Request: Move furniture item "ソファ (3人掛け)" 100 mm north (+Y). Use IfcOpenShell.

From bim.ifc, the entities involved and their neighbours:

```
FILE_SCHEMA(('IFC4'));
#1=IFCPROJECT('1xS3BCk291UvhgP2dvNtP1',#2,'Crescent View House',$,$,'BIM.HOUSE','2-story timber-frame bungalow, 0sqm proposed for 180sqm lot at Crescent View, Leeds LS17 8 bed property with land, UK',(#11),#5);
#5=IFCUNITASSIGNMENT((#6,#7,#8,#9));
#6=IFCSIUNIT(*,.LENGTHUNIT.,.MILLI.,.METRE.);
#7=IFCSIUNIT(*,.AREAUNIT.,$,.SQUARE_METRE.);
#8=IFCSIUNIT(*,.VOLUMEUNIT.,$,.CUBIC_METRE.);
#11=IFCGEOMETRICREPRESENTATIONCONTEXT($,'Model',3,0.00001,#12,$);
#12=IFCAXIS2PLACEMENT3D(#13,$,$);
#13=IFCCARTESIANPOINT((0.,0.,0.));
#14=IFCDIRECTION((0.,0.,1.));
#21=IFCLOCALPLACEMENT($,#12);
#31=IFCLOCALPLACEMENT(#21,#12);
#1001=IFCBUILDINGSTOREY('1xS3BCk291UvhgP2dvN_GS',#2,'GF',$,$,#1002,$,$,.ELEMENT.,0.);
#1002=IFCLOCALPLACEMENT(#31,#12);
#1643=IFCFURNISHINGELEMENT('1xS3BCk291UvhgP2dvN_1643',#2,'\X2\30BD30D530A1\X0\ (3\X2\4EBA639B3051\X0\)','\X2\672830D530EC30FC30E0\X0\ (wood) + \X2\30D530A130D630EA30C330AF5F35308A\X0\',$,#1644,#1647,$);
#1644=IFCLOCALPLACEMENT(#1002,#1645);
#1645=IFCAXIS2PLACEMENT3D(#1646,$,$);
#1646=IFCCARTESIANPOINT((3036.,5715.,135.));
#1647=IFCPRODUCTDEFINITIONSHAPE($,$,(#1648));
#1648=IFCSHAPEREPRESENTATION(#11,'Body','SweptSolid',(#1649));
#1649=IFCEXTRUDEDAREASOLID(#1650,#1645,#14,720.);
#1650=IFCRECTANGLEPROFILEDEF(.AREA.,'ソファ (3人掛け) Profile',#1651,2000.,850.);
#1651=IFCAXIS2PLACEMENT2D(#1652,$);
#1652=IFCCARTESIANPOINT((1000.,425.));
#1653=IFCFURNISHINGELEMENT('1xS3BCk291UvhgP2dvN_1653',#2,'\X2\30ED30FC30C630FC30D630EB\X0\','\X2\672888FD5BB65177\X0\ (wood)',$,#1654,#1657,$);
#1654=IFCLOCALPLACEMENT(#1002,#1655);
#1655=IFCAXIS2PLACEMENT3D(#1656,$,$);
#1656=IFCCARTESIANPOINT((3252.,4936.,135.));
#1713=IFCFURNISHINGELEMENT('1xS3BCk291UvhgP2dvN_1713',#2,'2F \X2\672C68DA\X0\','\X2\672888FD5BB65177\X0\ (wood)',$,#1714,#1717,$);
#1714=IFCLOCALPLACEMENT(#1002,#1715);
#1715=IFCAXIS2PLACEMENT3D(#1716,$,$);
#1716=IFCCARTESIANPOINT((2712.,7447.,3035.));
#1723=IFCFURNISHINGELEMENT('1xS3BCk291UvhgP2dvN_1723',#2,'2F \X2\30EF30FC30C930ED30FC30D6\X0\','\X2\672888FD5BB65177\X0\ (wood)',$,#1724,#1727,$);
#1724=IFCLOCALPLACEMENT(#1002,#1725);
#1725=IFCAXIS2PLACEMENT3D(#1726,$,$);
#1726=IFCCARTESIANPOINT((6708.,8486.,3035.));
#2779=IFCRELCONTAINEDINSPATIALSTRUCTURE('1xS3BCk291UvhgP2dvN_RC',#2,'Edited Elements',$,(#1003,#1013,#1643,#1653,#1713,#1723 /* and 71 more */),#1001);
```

```python
import ifcopenshell
import ifcopenshell.api.geometry
import ifcopenshell.util.placement
import ifcopenshell.util.unit

model = ifcopenshell.open("bim.ifc")
unit_scale = ifcopenshell.util.unit.calculate_unit_scale(model)

item = model.by_guid("1xS3BCk291UvhgP2dvN_1643")
matrix = ifcopenshell.util.placement.get_local_placement(item.ObjectPlacement)
matrix[1, 3] += 0.1 / unit_scale
ifcopenshell.api.geometry.edit_object_placement(model, product=item, matrix=matrix, is_si=False)

print(ifcopenshell.util.placement.get_local_placement(item.ObjectPlacement).round(3) + 0.0)

model.write("bim_updated.ifc")
```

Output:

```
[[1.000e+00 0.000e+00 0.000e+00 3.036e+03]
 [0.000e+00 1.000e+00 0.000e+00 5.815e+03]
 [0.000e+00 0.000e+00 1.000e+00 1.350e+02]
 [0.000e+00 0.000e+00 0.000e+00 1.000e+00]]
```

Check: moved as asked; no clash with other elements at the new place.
